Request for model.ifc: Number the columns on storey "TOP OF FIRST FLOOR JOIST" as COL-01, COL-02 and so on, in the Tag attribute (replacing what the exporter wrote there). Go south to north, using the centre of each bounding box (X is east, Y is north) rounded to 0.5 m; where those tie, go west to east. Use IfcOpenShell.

First a look at what the model holds.

```python
import ifcopenshell
import ifcopenshell.util.element
import ifcopenshell.util.placement

model = ifcopenshell.open("model.ifc")
print(model.schema)
storey = next(s for s in model.by_type("IfcBuildingStorey") if s.Name == "TOP OF FIRST FLOOR JOIST")
columns = [e for e in ifcopenshell.util.element.get_decomposition(storey) if e.is_a("IfcColumn")]
for e in sorted(columns, key=lambda e: e.id()):
    origin = ifcopenshell.util.placement.get_local_placement(e.ObjectPlacement)[:3, 3]
    print(e.id(), e.Tag, e.Name, origin.round(2) + 0.0, sep=" | ")
```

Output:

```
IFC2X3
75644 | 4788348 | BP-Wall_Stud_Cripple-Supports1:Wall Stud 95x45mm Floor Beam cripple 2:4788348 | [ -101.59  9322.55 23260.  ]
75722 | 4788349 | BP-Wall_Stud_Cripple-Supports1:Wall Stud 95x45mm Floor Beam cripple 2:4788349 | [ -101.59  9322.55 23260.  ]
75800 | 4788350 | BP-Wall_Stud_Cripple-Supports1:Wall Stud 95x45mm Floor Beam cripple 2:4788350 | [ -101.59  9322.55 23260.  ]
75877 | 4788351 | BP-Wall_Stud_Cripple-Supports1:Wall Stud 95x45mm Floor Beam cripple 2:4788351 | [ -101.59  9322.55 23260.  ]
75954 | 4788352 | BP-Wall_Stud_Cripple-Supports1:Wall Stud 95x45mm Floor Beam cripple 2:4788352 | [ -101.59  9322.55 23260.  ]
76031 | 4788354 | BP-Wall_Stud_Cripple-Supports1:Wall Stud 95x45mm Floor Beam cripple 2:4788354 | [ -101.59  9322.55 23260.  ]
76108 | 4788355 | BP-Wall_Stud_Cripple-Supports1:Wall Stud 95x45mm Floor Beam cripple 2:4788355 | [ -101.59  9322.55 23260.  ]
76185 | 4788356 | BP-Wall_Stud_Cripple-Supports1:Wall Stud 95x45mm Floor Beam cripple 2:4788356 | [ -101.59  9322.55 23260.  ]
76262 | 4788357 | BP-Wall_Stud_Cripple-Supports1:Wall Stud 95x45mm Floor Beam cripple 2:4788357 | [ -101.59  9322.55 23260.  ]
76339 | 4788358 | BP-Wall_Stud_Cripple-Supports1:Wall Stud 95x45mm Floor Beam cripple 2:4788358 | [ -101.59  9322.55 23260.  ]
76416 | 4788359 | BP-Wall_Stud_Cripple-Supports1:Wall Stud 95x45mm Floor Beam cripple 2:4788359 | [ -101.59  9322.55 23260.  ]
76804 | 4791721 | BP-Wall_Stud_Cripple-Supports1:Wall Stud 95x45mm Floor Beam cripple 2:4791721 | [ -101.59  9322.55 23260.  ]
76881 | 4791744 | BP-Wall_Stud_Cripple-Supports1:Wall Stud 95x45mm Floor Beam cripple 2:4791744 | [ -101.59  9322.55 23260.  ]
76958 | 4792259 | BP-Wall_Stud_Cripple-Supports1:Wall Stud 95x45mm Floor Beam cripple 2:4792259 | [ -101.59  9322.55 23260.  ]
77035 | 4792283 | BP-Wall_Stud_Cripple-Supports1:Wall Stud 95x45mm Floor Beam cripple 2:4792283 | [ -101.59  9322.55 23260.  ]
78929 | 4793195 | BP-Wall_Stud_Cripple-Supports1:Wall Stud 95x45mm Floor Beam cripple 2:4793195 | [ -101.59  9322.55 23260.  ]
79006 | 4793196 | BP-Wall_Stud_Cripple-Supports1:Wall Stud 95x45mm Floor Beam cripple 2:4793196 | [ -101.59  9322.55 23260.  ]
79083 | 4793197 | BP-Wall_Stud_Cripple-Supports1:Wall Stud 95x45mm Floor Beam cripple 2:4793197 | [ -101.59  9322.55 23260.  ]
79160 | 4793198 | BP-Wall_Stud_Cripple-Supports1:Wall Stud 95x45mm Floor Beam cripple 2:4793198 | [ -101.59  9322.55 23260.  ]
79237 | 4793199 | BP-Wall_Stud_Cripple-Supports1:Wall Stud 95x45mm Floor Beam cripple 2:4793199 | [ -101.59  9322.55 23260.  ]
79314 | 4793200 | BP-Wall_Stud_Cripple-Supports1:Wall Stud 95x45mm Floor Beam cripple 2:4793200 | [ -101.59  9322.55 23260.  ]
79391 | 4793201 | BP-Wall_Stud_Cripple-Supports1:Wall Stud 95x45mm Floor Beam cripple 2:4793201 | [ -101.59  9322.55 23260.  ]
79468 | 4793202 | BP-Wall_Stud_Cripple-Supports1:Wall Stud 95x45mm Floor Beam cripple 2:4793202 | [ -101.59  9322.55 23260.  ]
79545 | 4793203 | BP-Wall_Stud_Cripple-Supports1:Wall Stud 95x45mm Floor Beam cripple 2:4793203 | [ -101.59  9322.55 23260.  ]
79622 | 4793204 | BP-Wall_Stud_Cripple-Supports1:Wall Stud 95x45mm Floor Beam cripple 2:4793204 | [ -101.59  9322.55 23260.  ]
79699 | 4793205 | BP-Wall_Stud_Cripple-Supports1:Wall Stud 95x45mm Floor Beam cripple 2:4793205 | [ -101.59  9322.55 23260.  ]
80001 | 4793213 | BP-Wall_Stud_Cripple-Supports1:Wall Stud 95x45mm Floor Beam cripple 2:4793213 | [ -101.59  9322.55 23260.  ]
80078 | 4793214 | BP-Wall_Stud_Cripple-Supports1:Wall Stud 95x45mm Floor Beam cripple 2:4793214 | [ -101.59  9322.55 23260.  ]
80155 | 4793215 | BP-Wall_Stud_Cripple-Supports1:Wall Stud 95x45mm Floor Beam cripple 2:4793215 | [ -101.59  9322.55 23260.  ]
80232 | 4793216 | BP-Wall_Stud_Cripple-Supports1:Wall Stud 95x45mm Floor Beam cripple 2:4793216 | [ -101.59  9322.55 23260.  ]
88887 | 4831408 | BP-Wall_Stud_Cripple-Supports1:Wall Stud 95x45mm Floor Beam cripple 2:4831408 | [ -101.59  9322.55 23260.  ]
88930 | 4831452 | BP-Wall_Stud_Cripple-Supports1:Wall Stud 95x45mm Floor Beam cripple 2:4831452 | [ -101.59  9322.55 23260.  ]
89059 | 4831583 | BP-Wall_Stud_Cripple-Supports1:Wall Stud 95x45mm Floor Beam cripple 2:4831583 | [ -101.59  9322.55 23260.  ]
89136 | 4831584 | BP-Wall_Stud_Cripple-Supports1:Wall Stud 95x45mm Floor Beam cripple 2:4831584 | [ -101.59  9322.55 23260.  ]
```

```python
import ifcopenshell
import ifcopenshell.geom
import ifcopenshell.util.element
import ifcopenshell.util.shape

model = ifcopenshell.open("model.ifc")
settings = ifcopenshell.geom.settings()
settings.set("use-world-coords", True)


def centre(element):
    shape = ifcopenshell.geom.create_shape(settings, element)
    return ifcopenshell.util.shape.get_bbox_centroid(shape.geometry)


storey = next(s for s in model.by_type("IfcBuildingStorey") if s.Name == "TOP OF FIRST FLOOR JOIST")
columns = [e for e in ifcopenshell.util.element.get_decomposition(storey) if e.is_a("IfcColumn")]

# Insertion points can sit at a corner or the storey origin, so sort by the geometry (in metres).
centres = {e: centre(e) for e in columns}
columns.sort(key=lambda e: (round(centres[e][1] / 0.5), centres[e][0]))

for i, e in enumerate(columns, start=1):
    number = f"COL-{i:02d}"
    e.Tag = number
    print(e.id(), number)

model.write("model_updated.ifc")
```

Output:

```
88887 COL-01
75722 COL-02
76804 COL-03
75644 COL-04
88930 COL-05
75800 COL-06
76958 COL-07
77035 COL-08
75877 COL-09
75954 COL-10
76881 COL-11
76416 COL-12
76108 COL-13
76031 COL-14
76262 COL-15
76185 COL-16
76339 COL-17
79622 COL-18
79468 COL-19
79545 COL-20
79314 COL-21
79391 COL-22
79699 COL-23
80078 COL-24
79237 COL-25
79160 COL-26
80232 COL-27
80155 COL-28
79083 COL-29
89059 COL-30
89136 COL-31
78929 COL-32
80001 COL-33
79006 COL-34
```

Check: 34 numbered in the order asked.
